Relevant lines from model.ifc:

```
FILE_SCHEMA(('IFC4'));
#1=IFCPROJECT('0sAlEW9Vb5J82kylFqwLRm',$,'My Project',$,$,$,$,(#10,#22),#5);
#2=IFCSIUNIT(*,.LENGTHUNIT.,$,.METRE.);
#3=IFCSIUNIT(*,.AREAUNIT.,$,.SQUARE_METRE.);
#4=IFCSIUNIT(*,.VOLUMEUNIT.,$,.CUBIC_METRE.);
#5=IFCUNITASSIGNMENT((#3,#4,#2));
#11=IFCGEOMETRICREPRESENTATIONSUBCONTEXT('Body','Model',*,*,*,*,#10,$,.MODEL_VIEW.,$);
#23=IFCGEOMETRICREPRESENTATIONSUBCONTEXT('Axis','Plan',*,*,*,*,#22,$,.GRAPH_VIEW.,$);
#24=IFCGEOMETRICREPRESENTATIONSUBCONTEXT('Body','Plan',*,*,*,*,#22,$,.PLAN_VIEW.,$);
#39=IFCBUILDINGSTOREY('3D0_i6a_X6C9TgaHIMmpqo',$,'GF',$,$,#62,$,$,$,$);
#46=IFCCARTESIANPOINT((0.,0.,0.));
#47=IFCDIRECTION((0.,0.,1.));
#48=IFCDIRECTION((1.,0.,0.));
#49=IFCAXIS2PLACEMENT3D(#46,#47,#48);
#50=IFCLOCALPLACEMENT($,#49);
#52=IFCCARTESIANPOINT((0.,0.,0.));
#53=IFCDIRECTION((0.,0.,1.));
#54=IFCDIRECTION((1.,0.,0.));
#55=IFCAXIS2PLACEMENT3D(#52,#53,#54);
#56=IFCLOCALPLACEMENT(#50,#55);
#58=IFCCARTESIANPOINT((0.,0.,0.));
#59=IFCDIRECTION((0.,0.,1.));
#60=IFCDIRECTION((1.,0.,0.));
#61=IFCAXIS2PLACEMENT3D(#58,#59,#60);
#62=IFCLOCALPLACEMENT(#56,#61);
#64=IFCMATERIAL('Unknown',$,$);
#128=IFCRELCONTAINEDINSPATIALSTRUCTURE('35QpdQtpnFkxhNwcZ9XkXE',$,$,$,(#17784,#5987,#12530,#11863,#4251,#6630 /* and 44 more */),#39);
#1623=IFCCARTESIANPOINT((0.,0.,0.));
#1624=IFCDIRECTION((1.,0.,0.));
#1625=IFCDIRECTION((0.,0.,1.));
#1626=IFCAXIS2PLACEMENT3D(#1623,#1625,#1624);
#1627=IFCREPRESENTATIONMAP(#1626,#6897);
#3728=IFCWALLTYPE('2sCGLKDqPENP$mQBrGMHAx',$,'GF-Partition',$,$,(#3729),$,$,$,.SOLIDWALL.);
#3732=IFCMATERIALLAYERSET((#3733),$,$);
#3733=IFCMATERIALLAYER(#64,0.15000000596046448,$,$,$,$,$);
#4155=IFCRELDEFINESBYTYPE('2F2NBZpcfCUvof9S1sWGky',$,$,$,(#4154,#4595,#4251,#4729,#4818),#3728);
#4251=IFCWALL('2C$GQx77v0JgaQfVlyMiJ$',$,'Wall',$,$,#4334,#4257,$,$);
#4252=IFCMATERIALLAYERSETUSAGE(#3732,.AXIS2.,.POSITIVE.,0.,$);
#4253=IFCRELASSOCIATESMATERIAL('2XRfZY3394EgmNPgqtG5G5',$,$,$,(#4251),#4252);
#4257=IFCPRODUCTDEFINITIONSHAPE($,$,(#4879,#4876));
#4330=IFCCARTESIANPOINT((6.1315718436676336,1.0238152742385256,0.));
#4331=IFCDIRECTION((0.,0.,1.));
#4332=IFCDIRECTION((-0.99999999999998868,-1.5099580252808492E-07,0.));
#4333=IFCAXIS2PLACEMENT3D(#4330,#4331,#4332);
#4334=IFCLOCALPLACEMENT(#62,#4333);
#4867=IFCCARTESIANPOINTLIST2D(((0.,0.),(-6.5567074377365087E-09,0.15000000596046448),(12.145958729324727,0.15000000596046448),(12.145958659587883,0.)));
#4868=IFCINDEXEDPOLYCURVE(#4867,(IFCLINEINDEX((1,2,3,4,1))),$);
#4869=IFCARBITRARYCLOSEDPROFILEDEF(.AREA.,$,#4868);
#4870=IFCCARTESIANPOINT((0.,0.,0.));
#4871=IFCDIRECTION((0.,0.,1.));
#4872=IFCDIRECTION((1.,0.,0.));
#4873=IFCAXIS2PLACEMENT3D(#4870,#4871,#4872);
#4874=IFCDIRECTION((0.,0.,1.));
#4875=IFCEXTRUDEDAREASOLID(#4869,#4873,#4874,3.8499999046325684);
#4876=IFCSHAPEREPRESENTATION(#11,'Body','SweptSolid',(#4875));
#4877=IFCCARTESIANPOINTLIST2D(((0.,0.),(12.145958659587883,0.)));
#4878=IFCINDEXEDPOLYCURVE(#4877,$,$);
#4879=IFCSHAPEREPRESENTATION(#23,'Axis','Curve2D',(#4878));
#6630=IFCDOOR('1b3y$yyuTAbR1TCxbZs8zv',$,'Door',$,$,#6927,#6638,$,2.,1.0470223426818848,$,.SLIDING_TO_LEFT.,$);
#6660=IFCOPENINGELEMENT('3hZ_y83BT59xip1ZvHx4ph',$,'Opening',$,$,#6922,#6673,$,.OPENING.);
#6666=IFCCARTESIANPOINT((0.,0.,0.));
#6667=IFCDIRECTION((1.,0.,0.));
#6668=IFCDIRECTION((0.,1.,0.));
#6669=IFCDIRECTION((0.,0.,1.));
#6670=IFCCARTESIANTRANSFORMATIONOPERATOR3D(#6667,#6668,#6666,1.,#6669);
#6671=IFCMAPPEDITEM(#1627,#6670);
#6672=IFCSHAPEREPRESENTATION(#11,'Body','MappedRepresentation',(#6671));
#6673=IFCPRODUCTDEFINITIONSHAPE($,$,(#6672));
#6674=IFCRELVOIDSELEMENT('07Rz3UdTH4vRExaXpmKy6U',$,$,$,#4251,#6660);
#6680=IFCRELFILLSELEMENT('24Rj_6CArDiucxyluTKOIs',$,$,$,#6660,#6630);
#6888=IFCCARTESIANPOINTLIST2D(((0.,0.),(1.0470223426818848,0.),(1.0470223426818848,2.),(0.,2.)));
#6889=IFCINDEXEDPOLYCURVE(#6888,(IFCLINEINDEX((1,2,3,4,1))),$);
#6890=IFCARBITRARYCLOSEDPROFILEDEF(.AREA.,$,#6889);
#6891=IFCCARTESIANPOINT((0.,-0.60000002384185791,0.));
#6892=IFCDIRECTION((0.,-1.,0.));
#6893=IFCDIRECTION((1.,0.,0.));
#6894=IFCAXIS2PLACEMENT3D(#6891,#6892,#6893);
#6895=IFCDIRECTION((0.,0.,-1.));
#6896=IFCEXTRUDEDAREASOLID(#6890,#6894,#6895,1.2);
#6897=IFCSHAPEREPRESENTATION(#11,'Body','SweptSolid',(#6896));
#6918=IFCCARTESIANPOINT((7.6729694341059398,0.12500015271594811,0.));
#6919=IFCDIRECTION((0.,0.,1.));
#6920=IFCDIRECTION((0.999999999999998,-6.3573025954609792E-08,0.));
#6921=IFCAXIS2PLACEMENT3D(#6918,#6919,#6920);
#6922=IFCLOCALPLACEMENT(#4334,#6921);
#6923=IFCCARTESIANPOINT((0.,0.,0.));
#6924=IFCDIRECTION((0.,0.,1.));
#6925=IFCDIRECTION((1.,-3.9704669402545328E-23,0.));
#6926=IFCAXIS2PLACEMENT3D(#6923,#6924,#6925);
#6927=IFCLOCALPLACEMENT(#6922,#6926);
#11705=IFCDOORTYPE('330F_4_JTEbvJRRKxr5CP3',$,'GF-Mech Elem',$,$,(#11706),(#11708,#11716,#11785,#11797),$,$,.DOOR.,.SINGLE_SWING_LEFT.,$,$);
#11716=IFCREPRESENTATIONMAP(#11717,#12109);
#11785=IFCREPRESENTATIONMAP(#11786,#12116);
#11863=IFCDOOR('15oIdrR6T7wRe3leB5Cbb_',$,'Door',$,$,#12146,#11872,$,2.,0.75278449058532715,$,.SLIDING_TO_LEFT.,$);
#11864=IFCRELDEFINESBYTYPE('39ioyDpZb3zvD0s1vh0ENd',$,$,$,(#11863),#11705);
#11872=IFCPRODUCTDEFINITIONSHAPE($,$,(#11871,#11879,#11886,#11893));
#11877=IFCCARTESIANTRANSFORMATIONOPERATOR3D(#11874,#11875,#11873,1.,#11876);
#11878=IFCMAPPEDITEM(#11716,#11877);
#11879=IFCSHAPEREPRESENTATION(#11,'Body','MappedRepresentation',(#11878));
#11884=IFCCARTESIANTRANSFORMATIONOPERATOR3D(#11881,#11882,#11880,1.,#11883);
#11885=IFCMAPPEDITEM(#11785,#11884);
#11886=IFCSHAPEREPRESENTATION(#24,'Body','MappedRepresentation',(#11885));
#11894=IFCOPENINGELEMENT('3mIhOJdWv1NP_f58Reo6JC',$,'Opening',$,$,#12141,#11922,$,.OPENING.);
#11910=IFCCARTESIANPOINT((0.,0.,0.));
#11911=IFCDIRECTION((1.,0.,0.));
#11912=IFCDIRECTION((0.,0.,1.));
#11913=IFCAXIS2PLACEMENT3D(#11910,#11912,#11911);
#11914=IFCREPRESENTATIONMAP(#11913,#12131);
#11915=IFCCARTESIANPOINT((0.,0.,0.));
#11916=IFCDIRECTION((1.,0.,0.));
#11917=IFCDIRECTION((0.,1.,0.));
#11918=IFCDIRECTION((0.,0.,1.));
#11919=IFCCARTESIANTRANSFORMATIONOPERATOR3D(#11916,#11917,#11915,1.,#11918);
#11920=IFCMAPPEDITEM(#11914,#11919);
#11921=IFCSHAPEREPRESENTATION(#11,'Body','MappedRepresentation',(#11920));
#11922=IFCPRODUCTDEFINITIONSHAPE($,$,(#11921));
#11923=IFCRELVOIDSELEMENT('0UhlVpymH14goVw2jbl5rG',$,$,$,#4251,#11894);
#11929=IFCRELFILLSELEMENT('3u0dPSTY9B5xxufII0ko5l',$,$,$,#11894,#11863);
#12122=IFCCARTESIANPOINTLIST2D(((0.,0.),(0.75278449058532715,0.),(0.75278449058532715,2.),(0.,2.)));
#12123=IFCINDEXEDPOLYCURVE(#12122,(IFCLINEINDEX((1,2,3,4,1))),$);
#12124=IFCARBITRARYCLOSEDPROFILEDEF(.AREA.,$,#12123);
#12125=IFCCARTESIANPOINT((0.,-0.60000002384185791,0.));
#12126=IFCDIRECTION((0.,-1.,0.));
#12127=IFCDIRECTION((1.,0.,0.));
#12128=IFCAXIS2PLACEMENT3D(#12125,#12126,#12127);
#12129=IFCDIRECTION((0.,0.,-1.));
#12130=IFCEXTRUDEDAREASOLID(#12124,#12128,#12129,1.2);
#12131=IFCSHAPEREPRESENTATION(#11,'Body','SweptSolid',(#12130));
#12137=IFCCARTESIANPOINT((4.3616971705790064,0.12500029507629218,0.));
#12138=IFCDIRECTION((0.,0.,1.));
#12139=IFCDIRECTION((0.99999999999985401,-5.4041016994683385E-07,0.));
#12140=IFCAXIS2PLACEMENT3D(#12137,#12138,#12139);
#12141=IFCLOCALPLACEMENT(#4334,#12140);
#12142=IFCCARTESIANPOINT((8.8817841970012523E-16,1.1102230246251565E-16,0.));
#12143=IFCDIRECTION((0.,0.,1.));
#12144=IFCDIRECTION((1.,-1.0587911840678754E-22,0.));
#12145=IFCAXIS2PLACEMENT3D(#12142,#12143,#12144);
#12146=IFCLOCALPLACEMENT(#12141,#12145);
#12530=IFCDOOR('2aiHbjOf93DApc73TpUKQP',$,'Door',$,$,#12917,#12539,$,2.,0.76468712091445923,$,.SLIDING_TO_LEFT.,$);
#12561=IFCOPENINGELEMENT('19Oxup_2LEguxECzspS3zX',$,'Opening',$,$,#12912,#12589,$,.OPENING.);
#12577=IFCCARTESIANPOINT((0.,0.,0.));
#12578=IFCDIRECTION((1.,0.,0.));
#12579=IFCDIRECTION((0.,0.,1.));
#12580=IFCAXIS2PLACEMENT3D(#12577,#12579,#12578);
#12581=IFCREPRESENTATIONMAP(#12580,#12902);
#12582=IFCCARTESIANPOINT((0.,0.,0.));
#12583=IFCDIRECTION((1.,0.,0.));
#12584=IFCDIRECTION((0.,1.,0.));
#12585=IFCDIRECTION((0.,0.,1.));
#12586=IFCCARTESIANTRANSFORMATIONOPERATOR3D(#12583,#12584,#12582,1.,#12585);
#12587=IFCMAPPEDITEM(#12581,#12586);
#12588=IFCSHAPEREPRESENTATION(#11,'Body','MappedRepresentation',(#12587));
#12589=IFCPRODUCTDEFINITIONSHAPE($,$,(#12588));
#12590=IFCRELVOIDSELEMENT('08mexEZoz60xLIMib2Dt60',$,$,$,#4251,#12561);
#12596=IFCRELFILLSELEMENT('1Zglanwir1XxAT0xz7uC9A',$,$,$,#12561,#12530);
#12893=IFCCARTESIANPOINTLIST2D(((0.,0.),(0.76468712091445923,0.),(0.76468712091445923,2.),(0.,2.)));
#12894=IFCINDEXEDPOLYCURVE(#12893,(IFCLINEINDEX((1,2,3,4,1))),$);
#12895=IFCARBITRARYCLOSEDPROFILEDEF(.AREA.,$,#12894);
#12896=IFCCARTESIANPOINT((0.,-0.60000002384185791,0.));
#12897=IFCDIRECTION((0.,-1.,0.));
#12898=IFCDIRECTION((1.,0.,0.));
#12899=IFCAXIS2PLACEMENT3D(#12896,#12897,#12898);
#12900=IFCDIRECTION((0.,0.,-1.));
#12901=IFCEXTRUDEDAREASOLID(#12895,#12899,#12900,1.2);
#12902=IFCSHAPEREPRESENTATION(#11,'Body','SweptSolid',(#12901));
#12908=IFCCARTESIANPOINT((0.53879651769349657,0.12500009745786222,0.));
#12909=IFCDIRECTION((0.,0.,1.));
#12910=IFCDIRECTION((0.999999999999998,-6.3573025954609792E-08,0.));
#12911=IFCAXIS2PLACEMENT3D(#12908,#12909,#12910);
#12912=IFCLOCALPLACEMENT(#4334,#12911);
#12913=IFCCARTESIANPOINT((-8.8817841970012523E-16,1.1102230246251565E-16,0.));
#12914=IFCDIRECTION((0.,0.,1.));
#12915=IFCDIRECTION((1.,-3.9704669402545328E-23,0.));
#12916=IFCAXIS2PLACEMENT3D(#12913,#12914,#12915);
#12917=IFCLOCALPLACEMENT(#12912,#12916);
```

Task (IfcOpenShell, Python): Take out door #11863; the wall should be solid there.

```python
import ifcopenshell
import ifcopenshell.api.feature
import ifcopenshell.api.root
import ifcopenshell.geom
import ifcopenshell.util.shape

model = ifcopenshell.open("model.ifc")
settings = ifcopenshell.geom.settings()


def volume(element):
    """Net volume in cubic metres, openings subtracted."""
    shape = ifcopenshell.geom.create_shape(settings, element)
    return ifcopenshell.util.shape.get_volume(shape.geometry)


door = model.by_id(11863)
opening = door.FillsVoids[0].RelatingOpeningElement
wall = opening.VoidsElements[0].RelatingBuildingElement
before = volume(wall)

ifcopenshell.api.root.remove_product(model, product=door)
ifcopenshell.api.feature.remove_feature(model, feature=opening)

after = volume(wall)

print(f"wall volume {before:.3f} -> {after:.3f} m3")

model.write("model_updated.ifc")
```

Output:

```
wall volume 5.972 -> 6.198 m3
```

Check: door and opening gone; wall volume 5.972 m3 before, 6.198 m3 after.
